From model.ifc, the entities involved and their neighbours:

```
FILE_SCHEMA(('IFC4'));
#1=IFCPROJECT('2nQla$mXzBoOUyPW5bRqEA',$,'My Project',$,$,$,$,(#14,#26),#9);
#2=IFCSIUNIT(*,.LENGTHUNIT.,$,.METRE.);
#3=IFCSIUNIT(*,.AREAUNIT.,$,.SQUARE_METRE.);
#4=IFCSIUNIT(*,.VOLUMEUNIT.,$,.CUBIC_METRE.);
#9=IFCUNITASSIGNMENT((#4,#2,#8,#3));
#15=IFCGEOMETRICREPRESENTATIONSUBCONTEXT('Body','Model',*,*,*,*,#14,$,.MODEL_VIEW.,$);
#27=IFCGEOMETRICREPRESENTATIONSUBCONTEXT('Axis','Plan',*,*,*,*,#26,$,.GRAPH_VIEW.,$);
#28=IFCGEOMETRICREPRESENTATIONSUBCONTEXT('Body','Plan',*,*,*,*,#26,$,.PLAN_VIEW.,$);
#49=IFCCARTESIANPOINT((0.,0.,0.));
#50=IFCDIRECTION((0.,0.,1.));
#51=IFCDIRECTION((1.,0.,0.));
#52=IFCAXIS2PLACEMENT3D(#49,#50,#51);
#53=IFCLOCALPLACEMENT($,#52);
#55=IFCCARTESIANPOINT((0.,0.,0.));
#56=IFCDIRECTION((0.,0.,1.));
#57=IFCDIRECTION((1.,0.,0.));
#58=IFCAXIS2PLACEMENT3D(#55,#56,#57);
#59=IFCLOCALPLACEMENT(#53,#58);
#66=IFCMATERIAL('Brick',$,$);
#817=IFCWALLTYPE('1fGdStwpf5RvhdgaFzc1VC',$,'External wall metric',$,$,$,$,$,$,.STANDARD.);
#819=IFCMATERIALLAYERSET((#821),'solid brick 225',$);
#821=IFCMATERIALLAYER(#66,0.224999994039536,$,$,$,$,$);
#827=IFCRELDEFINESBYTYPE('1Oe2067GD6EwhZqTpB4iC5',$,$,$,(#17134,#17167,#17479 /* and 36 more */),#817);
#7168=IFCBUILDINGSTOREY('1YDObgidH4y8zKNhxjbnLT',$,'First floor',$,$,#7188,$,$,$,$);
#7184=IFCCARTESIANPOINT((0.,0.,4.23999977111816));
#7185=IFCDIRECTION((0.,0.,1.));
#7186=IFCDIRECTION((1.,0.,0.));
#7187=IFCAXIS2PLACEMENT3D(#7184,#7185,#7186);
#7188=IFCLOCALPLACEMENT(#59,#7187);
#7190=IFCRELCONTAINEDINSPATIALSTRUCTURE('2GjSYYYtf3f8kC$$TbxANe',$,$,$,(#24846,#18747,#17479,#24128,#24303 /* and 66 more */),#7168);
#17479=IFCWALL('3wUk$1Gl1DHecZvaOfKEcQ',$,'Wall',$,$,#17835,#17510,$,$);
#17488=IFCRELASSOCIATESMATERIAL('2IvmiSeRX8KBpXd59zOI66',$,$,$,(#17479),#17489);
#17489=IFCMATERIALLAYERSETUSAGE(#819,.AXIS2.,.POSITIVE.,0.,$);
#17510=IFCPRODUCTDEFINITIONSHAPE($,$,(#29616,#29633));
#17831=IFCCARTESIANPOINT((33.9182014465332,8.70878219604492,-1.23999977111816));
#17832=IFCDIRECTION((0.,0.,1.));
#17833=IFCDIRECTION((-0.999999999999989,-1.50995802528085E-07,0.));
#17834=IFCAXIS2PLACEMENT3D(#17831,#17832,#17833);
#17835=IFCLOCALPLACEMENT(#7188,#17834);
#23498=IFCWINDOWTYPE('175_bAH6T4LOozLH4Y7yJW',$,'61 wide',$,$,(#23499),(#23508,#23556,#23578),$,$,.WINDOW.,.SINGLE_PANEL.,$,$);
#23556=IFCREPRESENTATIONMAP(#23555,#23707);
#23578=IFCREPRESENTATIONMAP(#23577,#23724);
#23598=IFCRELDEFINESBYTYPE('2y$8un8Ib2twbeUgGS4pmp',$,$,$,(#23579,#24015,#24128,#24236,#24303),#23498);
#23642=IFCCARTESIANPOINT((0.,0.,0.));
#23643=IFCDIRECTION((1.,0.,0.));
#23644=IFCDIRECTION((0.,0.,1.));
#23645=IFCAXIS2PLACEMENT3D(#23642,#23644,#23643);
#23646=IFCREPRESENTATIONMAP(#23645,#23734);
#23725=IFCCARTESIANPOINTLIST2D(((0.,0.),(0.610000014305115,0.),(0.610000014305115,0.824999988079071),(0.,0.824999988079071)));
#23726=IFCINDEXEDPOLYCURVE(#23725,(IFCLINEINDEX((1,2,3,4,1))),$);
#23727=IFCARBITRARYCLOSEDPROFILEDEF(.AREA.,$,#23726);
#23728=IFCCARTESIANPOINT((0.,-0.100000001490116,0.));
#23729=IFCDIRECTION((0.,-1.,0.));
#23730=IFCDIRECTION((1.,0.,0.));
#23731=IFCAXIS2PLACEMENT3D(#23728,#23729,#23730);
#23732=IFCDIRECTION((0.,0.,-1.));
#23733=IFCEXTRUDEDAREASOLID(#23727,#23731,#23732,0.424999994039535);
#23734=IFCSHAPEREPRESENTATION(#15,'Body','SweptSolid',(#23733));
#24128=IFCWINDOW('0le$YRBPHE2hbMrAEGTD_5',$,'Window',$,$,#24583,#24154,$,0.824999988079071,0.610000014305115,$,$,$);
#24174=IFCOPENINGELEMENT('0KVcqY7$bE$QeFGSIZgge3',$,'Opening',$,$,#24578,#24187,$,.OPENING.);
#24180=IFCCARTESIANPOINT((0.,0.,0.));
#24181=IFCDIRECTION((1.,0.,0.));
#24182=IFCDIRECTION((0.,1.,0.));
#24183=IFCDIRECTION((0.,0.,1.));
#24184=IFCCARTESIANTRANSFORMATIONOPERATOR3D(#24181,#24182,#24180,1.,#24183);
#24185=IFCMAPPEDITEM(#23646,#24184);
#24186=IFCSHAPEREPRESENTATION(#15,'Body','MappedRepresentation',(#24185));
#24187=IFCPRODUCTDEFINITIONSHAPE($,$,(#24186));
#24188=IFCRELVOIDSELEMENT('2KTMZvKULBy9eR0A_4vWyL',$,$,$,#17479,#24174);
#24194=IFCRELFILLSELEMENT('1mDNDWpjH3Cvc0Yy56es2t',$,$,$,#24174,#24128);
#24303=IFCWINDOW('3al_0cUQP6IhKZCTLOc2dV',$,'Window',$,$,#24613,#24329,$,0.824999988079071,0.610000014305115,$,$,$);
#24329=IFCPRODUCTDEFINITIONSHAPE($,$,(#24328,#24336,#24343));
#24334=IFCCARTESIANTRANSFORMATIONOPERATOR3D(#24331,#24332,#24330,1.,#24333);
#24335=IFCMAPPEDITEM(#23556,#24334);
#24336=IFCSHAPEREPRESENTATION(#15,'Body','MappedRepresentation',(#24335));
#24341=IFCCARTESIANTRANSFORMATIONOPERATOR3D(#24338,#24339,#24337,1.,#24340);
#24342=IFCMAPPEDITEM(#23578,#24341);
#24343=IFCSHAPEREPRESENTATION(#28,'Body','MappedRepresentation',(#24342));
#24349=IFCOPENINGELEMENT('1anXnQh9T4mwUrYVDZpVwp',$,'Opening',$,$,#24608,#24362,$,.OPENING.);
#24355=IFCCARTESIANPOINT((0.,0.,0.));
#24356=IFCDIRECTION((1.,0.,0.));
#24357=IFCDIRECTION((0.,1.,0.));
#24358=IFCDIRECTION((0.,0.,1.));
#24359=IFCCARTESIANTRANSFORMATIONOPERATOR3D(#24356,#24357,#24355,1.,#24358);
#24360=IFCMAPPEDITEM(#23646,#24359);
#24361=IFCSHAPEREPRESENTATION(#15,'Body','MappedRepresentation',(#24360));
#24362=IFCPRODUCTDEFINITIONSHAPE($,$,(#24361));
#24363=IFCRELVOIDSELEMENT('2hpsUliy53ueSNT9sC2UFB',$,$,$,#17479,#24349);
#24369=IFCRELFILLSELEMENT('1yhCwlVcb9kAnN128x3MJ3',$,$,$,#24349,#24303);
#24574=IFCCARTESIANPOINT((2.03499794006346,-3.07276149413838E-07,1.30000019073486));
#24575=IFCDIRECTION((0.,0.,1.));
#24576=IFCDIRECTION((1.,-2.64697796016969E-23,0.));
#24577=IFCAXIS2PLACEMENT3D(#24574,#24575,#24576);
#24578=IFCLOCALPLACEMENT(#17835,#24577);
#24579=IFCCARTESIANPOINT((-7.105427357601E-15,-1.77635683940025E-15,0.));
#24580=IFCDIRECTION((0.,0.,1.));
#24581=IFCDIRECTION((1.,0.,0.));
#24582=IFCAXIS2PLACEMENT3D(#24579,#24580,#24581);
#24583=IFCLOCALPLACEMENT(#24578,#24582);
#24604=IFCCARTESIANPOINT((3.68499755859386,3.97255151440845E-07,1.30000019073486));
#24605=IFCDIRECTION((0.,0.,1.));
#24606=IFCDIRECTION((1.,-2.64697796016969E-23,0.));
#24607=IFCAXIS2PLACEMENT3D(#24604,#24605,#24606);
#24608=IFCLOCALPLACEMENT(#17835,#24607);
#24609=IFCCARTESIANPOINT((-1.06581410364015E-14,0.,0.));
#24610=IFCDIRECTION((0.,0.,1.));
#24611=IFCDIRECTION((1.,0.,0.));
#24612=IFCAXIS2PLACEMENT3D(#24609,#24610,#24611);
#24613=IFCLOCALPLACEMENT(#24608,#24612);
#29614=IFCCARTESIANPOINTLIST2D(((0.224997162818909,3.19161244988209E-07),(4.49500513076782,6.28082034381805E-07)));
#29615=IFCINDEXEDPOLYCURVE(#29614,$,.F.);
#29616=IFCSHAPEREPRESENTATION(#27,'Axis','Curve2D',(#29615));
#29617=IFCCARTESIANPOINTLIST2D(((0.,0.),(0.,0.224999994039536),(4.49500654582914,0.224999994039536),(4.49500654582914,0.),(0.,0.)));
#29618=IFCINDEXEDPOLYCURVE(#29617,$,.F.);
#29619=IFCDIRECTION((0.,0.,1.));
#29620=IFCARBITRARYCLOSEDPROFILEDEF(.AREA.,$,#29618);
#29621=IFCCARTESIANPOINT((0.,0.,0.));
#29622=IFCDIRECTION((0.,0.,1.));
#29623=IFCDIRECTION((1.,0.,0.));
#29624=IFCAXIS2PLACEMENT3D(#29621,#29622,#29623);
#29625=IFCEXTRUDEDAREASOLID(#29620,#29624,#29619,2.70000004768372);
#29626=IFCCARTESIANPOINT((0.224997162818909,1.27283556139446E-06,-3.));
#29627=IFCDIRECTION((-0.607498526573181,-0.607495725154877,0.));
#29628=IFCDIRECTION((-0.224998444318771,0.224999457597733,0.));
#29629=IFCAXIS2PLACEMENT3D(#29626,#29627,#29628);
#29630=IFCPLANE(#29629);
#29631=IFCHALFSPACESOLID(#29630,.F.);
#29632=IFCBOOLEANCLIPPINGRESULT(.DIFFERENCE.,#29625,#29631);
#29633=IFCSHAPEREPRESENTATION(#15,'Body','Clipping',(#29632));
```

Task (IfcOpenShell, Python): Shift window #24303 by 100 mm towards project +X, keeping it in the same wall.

```python
import ifcopenshell
import ifcopenshell.api.geometry
import ifcopenshell.util.placement
import ifcopenshell.util.unit

model = ifcopenshell.open("model.ifc")
unit_scale = ifcopenshell.util.unit.calculate_unit_scale(model)

window = model.by_guid("3al_0cUQP6IhKZCTLOc2dV")
opening = window.FillsVoids[0].RelatingOpeningElement
wall = opening.VoidsElements[0].RelatingBuildingElement

wall_matrix = ifcopenshell.util.placement.get_local_placement(wall.ObjectPlacement)
shift = wall_matrix[:3, 0] * -0.1 / unit_scale
before = ifcopenshell.util.placement.get_local_placement(window.ObjectPlacement)[:3, 3].copy()

# The window is placed relative to its opening, so it follows when the opening moves.
matrix = ifcopenshell.util.placement.get_local_placement(opening.ObjectPlacement)
matrix[:3, 3] += shift
ifcopenshell.api.geometry.edit_object_placement(
    model, product=opening, matrix=matrix, is_si=False, should_transform_children=True
)

after = ifcopenshell.util.placement.get_local_placement(window.ObjectPlacement)[:3, 3]
print("window moved by", (after - before).round(3) + 0.0)

model.write("model_v2.ifc")
```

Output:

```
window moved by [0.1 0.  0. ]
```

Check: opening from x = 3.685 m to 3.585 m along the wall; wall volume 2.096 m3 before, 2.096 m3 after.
